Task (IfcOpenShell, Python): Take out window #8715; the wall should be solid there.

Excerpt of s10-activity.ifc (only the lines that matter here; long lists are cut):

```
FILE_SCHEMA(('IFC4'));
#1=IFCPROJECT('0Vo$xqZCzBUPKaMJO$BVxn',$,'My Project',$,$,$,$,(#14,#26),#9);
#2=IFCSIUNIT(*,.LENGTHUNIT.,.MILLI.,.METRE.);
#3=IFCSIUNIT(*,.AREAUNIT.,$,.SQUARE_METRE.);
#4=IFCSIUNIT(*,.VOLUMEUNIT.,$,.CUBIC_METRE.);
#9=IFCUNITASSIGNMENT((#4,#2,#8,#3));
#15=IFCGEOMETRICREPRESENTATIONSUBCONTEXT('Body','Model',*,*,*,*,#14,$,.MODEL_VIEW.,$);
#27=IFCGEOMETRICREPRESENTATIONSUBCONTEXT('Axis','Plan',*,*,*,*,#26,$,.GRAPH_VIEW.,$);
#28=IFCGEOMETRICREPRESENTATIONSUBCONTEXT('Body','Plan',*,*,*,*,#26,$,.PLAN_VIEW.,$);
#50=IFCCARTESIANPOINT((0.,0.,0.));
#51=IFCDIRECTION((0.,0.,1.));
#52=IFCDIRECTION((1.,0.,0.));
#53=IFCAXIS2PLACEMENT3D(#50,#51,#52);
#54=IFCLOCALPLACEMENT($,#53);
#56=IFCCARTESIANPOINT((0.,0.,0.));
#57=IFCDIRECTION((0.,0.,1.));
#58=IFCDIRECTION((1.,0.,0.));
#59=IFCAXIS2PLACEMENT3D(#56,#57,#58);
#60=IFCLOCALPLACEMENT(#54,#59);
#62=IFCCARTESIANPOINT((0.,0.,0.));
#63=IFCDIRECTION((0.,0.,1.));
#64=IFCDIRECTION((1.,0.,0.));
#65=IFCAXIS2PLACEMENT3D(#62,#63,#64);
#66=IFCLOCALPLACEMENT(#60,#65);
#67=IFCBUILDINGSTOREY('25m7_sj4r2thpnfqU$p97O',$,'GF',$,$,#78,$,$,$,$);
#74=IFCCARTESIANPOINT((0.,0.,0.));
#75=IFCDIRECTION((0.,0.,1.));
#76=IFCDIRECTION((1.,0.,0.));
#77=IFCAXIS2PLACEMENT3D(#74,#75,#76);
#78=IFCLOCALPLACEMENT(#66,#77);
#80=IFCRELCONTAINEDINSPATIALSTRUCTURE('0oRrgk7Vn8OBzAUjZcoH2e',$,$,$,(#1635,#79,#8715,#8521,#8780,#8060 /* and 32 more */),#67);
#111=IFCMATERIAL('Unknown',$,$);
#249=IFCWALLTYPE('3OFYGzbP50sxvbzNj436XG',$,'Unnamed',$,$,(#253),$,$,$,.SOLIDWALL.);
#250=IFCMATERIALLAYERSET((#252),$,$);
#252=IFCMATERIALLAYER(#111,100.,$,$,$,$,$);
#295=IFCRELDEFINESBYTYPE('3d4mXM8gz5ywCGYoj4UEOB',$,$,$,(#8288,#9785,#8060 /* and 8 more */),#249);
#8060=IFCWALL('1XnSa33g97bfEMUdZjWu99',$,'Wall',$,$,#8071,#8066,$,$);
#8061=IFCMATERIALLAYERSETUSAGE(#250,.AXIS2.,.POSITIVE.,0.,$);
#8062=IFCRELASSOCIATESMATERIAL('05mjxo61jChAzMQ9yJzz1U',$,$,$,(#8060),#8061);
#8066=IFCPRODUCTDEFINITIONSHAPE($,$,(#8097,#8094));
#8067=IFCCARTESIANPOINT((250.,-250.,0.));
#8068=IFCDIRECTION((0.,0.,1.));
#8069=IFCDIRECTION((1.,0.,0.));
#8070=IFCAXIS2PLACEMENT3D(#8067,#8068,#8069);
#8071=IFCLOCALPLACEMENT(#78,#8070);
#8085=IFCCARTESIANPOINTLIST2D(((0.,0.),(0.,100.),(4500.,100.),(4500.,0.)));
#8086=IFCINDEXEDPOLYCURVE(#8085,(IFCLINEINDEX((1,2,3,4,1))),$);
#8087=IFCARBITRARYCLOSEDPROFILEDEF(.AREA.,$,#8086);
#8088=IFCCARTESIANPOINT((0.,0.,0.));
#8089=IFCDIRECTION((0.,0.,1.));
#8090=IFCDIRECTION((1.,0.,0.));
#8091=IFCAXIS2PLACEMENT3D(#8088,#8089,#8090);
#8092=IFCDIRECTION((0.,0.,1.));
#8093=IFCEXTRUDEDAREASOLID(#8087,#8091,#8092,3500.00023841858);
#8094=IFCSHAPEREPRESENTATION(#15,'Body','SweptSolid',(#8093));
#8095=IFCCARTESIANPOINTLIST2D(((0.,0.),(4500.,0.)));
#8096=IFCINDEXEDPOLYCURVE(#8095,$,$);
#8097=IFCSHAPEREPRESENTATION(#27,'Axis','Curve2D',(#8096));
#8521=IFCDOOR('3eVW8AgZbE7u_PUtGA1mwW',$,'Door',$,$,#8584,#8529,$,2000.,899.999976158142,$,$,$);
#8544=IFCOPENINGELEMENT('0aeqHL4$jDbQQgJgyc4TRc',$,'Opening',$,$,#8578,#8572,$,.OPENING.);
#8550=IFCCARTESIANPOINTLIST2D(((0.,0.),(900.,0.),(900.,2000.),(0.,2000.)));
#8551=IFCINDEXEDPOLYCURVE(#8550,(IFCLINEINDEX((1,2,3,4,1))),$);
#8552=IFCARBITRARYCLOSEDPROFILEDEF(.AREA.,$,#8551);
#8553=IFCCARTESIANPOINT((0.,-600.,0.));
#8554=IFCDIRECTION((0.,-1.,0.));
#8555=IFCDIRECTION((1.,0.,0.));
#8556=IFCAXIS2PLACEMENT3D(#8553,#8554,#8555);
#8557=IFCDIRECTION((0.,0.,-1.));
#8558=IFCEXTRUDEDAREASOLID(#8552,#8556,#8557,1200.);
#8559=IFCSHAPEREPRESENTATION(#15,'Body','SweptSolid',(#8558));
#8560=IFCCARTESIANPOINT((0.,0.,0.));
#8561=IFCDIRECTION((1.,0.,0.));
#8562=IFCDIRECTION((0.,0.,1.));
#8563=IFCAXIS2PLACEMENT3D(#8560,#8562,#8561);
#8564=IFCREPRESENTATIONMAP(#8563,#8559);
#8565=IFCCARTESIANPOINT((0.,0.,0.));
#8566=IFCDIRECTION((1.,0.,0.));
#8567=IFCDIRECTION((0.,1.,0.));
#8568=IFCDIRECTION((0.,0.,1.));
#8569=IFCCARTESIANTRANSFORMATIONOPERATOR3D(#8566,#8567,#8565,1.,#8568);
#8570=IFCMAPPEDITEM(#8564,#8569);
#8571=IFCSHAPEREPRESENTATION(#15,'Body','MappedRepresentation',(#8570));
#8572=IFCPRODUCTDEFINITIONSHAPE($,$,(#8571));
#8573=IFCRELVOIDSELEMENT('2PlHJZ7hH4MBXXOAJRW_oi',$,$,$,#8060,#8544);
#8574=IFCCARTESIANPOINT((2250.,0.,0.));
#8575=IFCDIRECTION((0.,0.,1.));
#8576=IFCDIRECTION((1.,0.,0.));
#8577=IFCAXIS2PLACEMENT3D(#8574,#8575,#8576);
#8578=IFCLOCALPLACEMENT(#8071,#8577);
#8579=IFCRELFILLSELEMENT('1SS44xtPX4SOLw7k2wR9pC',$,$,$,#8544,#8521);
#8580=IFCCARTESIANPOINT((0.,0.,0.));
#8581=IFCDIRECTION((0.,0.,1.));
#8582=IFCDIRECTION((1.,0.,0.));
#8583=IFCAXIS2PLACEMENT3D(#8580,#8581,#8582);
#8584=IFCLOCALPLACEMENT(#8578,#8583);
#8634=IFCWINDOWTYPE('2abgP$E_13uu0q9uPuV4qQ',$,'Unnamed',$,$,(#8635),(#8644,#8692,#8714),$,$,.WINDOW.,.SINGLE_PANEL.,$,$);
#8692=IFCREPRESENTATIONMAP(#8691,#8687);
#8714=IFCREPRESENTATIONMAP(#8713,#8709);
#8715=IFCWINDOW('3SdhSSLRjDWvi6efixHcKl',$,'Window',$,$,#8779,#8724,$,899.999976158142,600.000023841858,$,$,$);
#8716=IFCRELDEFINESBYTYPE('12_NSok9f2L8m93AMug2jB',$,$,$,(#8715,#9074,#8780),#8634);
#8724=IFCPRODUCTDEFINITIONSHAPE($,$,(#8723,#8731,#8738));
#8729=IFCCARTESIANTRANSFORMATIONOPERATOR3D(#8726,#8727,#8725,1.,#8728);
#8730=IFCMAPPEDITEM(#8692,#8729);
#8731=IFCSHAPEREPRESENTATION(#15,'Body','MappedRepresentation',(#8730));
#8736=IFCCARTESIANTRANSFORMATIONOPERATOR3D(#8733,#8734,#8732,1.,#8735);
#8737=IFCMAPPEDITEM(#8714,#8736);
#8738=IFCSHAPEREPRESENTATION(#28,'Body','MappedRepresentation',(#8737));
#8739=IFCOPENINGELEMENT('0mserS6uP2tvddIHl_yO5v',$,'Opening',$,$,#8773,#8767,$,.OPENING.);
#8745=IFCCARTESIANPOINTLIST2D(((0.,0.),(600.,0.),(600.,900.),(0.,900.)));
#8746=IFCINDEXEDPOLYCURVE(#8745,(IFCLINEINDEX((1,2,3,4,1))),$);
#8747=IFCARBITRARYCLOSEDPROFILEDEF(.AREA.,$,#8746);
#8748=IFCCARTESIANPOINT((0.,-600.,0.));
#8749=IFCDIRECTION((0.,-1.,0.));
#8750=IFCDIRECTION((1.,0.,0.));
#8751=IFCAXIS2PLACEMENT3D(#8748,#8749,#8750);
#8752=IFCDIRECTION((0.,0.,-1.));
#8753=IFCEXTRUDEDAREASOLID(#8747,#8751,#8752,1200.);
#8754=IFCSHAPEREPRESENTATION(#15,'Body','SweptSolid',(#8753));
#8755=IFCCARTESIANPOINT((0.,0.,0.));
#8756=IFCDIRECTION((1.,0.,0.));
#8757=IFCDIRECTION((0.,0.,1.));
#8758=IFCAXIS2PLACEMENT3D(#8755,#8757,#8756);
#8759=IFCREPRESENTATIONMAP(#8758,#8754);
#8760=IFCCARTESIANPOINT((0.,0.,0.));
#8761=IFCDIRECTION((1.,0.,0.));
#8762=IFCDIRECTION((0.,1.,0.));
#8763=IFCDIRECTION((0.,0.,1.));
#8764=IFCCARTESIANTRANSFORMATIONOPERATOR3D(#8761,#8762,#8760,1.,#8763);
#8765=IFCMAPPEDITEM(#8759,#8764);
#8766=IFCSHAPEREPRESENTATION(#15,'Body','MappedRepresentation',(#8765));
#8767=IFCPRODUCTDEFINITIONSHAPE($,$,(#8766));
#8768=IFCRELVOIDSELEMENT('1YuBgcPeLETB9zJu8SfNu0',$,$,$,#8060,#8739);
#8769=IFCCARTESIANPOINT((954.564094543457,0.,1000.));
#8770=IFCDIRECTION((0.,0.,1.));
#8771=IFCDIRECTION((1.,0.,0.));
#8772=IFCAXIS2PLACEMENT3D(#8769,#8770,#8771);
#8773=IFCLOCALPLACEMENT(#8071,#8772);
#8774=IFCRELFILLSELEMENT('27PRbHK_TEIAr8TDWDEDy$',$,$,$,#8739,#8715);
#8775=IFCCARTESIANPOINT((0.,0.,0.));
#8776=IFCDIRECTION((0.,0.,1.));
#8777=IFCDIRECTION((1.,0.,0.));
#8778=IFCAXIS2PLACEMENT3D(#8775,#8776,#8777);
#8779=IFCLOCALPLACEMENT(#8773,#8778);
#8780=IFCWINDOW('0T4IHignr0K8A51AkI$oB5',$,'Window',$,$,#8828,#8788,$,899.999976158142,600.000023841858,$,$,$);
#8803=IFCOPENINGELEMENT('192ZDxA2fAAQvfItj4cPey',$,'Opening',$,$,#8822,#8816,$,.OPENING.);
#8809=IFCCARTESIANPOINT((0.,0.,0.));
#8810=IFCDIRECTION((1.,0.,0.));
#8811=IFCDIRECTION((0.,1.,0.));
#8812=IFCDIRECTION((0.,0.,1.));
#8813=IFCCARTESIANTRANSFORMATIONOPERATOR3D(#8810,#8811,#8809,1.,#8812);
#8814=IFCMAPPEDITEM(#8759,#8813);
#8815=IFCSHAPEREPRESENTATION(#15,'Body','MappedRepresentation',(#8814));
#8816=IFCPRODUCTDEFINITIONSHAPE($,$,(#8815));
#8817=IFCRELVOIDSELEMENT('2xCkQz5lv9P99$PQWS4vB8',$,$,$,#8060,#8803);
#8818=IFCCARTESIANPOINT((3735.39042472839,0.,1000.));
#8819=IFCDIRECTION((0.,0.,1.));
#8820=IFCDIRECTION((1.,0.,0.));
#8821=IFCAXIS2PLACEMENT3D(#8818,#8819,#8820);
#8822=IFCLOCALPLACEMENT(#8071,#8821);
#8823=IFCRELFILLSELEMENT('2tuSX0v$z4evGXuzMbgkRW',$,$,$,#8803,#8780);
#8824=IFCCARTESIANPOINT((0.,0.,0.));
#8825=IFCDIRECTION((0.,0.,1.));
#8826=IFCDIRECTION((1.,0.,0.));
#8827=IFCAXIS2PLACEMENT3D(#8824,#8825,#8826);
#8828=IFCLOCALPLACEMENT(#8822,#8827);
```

```python
import ifcopenshell
import ifcopenshell.api.feature
import ifcopenshell.api.root
import ifcopenshell.geom
import ifcopenshell.util.shape

model = ifcopenshell.open("s10-activity.ifc")
settings = ifcopenshell.geom.settings()


def volume(element):
    """Net volume in cubic metres, openings subtracted."""
    shape = ifcopenshell.geom.create_shape(settings, element)
    return ifcopenshell.util.shape.get_volume(shape.geometry)


window = model.by_guid("3SdhSSLRjDWvi6efixHcKl")
opening = window.FillsVoids[0].RelatingOpeningElement
wall = opening.VoidsElements[0].RelatingBuildingElement
before = volume(wall)

ifcopenshell.api.root.remove_product(model, product=window)
ifcopenshell.api.feature.remove_feature(model, feature=opening)

after = volume(wall)

print(f"wall volume {before:.3f} -> {after:.3f} m3")

model.write("s10-activity_v2.ifc")
```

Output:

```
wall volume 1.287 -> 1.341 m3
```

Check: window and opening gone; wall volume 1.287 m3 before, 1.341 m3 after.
